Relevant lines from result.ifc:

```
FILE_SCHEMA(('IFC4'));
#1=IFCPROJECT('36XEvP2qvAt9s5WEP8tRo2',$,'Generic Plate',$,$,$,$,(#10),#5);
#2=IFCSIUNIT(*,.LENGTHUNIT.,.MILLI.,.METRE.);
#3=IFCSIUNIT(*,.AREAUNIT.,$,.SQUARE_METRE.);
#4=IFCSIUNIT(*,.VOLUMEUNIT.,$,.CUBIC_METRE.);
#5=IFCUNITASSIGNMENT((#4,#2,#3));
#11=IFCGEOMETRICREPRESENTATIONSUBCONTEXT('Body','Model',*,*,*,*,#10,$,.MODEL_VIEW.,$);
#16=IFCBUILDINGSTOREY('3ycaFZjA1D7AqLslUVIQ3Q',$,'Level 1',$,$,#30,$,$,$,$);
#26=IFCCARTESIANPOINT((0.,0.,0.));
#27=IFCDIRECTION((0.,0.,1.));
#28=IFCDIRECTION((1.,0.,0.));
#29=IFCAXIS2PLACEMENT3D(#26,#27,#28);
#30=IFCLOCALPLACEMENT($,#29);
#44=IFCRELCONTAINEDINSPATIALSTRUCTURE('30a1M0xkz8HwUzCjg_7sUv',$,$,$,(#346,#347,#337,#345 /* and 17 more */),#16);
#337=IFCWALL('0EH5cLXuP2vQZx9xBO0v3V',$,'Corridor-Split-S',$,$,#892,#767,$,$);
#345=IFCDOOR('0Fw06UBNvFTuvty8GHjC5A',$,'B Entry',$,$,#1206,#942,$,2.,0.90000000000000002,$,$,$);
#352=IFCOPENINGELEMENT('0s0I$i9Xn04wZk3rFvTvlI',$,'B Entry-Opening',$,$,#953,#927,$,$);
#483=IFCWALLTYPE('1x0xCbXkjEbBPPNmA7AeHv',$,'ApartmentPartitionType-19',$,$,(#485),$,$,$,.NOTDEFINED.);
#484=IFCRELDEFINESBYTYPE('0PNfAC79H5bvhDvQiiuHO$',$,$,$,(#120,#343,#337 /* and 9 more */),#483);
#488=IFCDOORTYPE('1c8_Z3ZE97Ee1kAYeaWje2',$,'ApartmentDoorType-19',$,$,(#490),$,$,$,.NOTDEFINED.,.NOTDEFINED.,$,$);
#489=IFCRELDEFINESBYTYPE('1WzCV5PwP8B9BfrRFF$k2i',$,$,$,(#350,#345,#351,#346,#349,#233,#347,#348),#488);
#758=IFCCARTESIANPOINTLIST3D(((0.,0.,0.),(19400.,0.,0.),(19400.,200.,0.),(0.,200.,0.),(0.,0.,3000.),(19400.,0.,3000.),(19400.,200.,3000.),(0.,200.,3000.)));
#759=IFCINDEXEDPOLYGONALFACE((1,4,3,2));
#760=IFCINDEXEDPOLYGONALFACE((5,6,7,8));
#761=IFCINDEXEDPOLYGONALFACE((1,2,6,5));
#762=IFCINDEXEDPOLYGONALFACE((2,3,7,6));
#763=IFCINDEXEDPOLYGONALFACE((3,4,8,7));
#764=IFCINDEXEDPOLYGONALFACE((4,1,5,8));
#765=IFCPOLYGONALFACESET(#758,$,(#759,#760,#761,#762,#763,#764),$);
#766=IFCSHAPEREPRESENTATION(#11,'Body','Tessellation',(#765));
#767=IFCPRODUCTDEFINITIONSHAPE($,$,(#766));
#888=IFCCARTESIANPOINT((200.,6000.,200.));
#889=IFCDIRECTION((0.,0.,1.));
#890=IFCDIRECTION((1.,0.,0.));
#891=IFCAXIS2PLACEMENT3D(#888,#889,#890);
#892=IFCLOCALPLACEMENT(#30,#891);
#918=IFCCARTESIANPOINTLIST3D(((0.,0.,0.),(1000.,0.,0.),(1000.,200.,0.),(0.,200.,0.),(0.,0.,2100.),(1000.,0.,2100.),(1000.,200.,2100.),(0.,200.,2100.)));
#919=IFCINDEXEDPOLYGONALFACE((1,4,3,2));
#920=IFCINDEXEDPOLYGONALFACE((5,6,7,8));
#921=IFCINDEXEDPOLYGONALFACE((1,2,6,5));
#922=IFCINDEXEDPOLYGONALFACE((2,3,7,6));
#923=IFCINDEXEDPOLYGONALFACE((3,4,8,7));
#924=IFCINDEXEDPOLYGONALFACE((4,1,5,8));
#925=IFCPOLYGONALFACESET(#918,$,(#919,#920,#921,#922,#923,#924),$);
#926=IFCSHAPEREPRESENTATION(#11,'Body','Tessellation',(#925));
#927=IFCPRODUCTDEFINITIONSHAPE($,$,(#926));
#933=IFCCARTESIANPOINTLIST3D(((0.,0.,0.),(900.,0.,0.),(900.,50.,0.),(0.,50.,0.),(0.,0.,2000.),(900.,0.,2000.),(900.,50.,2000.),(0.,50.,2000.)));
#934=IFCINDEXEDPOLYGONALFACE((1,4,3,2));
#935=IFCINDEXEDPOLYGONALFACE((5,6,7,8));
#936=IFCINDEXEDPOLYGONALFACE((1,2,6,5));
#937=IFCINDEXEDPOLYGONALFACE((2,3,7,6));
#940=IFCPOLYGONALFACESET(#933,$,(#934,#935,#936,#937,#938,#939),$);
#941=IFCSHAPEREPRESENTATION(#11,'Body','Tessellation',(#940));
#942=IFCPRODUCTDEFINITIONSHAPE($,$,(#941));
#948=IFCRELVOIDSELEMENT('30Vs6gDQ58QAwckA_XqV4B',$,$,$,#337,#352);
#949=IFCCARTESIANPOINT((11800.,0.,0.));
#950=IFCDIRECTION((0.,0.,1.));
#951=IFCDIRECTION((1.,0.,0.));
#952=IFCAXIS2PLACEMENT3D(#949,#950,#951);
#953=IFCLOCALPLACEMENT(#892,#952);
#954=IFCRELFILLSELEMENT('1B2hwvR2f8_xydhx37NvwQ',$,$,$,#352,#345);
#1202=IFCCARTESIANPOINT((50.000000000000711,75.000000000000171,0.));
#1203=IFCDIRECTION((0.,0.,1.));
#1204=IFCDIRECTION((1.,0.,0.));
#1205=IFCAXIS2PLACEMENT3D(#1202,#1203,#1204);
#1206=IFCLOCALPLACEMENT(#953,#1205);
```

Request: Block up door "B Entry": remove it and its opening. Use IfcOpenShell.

```python
import ifcopenshell
import ifcopenshell.api.feature
import ifcopenshell.api.root
import ifcopenshell.geom
import ifcopenshell.util.shape

model = ifcopenshell.open("result.ifc")
settings = ifcopenshell.geom.settings()


def volume(element):
    """Net volume in cubic metres, openings subtracted."""
    shape = ifcopenshell.geom.create_shape(settings, element)
    return ifcopenshell.util.shape.get_volume(shape.geometry)


door = model.by_guid("0Fw06UBNvFTuvty8GHjC5A")
opening = door.FillsVoids[0].RelatingOpeningElement
wall = opening.VoidsElements[0].RelatingBuildingElement
before = volume(wall)

ifcopenshell.api.root.remove_product(model, product=door)
ifcopenshell.api.feature.remove_feature(model, feature=opening)

after = volume(wall)

print(f"wall volume {before:.3f} -> {after:.3f} m3")

model.write("result_rev.ifc")
```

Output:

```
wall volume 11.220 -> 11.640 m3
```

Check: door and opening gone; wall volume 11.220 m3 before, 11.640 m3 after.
